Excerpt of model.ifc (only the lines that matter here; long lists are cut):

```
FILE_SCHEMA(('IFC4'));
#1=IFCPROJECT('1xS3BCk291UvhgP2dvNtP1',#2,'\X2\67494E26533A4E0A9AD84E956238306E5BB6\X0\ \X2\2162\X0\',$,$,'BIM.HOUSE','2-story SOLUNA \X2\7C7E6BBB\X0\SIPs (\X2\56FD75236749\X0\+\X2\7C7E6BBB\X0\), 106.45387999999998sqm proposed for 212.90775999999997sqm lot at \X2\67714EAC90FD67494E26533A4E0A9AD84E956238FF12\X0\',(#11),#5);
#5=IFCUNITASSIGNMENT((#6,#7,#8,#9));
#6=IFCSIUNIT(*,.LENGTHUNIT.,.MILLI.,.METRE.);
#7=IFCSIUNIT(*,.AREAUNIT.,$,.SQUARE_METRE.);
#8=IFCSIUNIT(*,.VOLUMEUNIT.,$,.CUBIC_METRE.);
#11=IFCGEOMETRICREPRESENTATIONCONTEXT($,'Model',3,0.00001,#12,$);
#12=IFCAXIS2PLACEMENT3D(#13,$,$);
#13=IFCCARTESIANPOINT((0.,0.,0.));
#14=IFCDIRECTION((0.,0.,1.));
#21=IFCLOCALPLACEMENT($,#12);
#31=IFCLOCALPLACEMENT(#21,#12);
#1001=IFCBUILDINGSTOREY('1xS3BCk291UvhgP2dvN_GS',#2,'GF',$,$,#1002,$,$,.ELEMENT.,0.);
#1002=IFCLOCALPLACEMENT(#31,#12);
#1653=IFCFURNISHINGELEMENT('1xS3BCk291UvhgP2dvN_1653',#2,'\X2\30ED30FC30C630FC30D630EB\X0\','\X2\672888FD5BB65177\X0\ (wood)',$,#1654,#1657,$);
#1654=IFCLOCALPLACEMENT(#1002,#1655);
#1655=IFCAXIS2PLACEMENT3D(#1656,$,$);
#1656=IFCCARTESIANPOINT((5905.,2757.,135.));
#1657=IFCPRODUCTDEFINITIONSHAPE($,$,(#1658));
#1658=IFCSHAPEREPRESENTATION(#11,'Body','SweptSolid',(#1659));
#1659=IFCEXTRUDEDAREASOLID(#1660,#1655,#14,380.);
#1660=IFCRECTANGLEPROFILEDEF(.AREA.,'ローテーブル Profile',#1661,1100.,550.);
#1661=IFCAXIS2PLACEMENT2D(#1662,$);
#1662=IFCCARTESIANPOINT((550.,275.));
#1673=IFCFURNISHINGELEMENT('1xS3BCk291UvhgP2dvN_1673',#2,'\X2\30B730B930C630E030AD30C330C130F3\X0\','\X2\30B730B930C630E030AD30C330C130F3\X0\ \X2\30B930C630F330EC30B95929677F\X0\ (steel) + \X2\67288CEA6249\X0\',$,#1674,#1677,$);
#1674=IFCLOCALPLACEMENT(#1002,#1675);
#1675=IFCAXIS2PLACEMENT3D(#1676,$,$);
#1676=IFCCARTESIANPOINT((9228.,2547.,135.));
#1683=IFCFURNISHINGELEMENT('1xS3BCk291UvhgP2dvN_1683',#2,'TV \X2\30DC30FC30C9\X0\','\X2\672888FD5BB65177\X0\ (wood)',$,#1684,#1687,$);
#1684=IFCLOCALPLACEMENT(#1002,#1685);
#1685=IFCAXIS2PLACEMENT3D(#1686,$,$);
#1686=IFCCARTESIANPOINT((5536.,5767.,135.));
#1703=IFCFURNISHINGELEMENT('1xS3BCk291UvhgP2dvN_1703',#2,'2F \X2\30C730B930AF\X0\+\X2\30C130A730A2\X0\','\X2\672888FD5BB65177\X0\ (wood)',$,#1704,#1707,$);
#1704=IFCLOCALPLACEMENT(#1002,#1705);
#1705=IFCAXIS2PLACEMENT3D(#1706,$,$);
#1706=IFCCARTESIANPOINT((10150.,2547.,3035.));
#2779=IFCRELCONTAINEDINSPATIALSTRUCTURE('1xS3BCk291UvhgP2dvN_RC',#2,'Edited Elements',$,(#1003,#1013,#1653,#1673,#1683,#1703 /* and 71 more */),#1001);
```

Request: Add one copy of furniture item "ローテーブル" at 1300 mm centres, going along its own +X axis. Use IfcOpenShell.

```python
import ifcopenshell
import ifcopenshell.api.geometry
import ifcopenshell.api.root
import ifcopenshell.util.element
import ifcopenshell.util.placement

model = ifcopenshell.open("model.ifc")


def reuse_history(source, copy):
    """copy_class also copies each property set's owner history, people and application; keep the originals."""
    for rel in copy.IsDefinedBy:
        if rel.is_a("IfcRelDefinesByProperties") and (history := rel.RelatingPropertyDefinition.OwnerHistory):
            rel.RelatingPropertyDefinition.OwnerHistory = source.OwnerHistory
            ifcopenshell.util.element.remove_deep2(model, history)


source = model.by_id(1653)
base = ifcopenshell.util.placement.get_local_placement(source.ObjectPlacement)
step = base[:3, 0] * 1300.0

for i in range(1, 2):
    copy = ifcopenshell.api.root.copy_class(model, product=source)
    copy.Representation = ifcopenshell.util.element.copy_deep(
        model, source.Representation, exclude=["IfcGeometricRepresentationContext", "IfcRepresentationMap"]
    )
    reuse_history(source, copy)
    matrix = base.copy()
    matrix[:3, 3] += i * step
    print("added at", matrix[:3, 3].round(3) + 0.0)
    ifcopenshell.api.geometry.edit_object_placement(model, product=copy, matrix=matrix, is_si=False)

model.write("model_rev.ifc")
```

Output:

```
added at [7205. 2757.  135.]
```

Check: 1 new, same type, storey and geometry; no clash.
